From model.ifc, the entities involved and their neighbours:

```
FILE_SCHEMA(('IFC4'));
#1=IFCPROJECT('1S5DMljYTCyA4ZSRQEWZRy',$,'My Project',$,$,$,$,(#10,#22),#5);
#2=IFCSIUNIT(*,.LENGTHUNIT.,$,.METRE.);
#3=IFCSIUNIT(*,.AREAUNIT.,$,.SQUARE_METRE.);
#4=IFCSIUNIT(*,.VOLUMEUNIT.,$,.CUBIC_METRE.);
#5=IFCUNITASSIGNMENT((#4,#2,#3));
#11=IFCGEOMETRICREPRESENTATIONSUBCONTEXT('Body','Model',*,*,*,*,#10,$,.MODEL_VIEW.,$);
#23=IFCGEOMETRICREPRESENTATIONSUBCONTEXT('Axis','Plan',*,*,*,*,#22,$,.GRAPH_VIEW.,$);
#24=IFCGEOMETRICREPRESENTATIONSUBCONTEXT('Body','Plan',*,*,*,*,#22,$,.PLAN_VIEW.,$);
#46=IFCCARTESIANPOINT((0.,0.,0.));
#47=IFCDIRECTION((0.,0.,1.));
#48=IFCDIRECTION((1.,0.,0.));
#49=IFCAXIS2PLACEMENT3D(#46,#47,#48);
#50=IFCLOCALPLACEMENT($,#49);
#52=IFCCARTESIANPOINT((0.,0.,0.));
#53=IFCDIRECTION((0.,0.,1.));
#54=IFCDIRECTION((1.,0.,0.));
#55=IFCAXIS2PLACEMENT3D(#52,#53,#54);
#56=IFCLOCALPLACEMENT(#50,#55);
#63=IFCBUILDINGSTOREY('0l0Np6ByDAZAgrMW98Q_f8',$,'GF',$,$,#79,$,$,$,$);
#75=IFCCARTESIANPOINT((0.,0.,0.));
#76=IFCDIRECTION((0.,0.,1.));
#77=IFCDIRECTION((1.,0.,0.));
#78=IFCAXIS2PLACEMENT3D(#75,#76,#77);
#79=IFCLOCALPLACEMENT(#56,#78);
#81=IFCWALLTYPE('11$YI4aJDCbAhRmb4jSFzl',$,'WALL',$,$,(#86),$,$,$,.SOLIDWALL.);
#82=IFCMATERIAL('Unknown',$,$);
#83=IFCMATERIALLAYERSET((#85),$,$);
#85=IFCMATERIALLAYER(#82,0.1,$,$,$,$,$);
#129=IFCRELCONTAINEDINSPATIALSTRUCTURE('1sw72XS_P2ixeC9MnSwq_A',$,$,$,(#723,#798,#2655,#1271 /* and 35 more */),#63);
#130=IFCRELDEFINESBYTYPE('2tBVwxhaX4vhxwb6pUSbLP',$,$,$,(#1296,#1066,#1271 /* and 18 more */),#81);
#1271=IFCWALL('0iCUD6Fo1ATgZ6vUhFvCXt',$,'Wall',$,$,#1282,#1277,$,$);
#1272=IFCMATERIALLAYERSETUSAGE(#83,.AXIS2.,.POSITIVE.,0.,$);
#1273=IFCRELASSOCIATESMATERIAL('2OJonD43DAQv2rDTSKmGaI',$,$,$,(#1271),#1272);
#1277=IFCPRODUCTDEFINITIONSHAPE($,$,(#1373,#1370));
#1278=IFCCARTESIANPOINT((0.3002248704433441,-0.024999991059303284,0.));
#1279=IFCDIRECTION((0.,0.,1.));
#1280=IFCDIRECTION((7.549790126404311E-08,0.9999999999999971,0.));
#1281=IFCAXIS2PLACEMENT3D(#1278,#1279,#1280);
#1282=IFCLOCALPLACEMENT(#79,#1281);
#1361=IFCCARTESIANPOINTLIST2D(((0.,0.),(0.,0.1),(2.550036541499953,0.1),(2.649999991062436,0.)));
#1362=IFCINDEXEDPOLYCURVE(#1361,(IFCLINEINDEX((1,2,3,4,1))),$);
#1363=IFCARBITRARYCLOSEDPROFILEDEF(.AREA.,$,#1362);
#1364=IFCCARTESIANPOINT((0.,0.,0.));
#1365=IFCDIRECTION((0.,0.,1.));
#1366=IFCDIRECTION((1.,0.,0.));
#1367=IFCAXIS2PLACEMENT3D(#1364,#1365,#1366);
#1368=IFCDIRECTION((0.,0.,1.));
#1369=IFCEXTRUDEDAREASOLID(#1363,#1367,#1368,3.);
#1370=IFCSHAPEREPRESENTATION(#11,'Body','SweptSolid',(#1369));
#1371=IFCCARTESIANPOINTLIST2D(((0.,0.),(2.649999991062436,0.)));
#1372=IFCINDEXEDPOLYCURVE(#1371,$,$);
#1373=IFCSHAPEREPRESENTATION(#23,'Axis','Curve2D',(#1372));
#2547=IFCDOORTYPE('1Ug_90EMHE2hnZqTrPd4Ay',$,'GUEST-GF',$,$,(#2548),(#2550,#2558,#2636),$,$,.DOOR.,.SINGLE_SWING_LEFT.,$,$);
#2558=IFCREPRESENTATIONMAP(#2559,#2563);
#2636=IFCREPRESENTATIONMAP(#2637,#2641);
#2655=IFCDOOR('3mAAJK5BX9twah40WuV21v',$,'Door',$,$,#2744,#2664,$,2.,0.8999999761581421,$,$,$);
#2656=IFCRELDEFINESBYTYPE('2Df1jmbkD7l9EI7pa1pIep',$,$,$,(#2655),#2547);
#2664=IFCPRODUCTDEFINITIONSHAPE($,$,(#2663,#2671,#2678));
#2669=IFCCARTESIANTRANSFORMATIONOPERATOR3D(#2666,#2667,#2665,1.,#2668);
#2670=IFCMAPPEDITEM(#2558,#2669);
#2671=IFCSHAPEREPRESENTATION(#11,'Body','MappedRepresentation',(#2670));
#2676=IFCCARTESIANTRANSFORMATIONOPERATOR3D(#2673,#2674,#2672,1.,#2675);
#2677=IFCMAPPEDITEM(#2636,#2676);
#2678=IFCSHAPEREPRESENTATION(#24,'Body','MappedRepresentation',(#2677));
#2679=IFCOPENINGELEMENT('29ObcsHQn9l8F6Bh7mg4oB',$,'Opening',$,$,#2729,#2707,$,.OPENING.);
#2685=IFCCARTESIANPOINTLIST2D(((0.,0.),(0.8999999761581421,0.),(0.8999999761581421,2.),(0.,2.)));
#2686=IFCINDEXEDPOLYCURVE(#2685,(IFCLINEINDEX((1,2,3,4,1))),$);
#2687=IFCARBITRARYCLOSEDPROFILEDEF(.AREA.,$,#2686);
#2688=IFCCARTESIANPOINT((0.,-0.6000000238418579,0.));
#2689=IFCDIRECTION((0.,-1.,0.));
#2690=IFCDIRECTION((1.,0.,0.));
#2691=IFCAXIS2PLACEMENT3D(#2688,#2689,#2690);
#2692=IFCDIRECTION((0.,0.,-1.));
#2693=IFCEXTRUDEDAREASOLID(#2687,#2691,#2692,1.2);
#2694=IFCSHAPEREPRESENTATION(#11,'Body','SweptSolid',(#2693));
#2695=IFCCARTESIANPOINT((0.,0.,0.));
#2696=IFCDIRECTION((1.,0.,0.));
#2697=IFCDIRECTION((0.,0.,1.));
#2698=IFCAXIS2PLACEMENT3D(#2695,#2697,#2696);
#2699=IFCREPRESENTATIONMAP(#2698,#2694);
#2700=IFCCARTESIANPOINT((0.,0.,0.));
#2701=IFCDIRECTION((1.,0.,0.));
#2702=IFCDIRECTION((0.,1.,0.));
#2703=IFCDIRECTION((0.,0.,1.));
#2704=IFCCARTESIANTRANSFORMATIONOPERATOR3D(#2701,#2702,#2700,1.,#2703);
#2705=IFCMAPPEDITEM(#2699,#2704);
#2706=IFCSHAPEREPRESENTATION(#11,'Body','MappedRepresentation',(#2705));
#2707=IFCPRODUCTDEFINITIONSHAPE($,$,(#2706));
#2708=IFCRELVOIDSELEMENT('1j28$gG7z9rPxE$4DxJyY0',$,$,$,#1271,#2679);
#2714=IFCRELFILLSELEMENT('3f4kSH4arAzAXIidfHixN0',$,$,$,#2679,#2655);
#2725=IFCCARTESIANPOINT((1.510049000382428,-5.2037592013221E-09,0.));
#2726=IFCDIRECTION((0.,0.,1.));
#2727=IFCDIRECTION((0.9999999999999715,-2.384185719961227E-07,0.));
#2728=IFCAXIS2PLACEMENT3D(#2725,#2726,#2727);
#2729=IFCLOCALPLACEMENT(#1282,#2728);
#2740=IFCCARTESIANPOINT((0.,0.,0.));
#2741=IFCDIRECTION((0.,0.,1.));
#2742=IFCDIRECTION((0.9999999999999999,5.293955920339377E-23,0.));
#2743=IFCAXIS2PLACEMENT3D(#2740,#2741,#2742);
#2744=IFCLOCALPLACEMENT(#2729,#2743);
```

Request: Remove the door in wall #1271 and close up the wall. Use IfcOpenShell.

```python
import ifcopenshell
import ifcopenshell.api.feature
import ifcopenshell.api.root
import ifcopenshell.geom
import ifcopenshell.util.shape

model = ifcopenshell.open("model.ifc")
settings = ifcopenshell.geom.settings()


def volume(element):
    """Net volume in cubic metres, openings subtracted."""
    shape = ifcopenshell.geom.create_shape(settings, element)
    return ifcopenshell.util.shape.get_volume(shape.geometry)


door = model.by_id(2655)
opening = door.FillsVoids[0].RelatingOpeningElement
wall = opening.VoidsElements[0].RelatingBuildingElement
before = volume(wall)

ifcopenshell.api.root.remove_product(model, product=door)
ifcopenshell.api.feature.remove_feature(model, feature=opening)

after = volume(wall)

print(f"wall volume {before:.3f} -> {after:.3f} m3")

model.write("model_v2.ifc")
```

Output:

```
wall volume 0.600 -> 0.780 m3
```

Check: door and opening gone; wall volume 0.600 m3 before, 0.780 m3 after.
